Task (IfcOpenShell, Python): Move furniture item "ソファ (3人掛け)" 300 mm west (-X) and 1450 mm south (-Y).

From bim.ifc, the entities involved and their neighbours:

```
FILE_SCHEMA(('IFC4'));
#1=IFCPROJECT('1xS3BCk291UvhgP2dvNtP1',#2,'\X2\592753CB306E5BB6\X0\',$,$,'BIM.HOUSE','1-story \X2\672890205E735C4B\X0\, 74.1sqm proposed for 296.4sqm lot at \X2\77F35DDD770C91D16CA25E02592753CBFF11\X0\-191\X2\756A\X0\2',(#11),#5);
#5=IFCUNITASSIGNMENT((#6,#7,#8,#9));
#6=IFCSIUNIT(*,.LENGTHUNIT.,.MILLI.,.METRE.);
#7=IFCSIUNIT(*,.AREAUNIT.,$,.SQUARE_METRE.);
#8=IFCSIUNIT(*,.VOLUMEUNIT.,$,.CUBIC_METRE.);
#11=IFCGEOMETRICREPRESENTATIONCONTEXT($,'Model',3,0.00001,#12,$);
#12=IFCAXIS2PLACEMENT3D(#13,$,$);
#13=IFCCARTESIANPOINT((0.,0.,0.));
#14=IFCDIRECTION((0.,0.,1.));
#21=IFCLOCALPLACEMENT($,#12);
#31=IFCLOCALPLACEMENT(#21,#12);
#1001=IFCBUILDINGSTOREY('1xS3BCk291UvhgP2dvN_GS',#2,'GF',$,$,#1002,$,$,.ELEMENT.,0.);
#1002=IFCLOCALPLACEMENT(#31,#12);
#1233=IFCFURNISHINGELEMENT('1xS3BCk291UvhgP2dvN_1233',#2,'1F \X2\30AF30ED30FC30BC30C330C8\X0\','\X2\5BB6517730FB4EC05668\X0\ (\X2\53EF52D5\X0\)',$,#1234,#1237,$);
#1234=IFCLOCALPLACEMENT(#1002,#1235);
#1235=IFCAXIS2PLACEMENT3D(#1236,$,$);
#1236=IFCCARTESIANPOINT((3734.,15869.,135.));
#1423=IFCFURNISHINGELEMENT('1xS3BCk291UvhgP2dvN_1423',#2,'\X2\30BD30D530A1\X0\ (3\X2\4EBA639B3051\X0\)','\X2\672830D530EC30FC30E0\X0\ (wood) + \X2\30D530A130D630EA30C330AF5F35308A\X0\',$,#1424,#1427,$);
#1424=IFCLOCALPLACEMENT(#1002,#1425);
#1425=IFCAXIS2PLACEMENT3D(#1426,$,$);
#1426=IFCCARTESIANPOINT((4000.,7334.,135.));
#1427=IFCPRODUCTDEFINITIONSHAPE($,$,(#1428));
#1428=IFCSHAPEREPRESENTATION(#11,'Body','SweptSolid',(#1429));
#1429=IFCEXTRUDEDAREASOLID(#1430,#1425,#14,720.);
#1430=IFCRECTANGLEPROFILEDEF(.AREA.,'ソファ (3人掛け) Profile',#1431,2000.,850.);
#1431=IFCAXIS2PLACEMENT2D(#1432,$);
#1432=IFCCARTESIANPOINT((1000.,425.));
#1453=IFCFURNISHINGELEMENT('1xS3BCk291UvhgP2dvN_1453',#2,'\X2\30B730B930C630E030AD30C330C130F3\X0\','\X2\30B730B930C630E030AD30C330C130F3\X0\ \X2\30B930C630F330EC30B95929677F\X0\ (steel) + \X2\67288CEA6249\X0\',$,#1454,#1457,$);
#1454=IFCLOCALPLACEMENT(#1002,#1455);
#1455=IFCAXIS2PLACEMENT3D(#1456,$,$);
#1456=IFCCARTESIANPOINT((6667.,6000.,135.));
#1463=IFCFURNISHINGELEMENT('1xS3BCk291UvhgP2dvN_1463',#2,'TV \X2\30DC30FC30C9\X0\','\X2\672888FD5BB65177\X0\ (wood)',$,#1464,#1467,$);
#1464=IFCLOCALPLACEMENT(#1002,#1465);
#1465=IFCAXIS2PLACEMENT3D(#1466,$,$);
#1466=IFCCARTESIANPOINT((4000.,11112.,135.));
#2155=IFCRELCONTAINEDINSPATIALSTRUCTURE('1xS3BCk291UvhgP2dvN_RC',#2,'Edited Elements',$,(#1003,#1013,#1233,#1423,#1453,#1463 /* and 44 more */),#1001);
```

```python
import ifcopenshell
import ifcopenshell.api.geometry
import ifcopenshell.util.placement

model = ifcopenshell.open("bim.ifc")

item = model.by_id(1423)
matrix = ifcopenshell.util.placement.get_local_placement(item.ObjectPlacement)
matrix[0, 3] -= 300.0
matrix[1, 3] -= 1450.0
ifcopenshell.api.geometry.edit_object_placement(model, product=item, matrix=matrix, is_si=False)

print(ifcopenshell.util.placement.get_local_placement(item.ObjectPlacement).round(3) + 0.0)

model.write("bim_rev.ifc")
```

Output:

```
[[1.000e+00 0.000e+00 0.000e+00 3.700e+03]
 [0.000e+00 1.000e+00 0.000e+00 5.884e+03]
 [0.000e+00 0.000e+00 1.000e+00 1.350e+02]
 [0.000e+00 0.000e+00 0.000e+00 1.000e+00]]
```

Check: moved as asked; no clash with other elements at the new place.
